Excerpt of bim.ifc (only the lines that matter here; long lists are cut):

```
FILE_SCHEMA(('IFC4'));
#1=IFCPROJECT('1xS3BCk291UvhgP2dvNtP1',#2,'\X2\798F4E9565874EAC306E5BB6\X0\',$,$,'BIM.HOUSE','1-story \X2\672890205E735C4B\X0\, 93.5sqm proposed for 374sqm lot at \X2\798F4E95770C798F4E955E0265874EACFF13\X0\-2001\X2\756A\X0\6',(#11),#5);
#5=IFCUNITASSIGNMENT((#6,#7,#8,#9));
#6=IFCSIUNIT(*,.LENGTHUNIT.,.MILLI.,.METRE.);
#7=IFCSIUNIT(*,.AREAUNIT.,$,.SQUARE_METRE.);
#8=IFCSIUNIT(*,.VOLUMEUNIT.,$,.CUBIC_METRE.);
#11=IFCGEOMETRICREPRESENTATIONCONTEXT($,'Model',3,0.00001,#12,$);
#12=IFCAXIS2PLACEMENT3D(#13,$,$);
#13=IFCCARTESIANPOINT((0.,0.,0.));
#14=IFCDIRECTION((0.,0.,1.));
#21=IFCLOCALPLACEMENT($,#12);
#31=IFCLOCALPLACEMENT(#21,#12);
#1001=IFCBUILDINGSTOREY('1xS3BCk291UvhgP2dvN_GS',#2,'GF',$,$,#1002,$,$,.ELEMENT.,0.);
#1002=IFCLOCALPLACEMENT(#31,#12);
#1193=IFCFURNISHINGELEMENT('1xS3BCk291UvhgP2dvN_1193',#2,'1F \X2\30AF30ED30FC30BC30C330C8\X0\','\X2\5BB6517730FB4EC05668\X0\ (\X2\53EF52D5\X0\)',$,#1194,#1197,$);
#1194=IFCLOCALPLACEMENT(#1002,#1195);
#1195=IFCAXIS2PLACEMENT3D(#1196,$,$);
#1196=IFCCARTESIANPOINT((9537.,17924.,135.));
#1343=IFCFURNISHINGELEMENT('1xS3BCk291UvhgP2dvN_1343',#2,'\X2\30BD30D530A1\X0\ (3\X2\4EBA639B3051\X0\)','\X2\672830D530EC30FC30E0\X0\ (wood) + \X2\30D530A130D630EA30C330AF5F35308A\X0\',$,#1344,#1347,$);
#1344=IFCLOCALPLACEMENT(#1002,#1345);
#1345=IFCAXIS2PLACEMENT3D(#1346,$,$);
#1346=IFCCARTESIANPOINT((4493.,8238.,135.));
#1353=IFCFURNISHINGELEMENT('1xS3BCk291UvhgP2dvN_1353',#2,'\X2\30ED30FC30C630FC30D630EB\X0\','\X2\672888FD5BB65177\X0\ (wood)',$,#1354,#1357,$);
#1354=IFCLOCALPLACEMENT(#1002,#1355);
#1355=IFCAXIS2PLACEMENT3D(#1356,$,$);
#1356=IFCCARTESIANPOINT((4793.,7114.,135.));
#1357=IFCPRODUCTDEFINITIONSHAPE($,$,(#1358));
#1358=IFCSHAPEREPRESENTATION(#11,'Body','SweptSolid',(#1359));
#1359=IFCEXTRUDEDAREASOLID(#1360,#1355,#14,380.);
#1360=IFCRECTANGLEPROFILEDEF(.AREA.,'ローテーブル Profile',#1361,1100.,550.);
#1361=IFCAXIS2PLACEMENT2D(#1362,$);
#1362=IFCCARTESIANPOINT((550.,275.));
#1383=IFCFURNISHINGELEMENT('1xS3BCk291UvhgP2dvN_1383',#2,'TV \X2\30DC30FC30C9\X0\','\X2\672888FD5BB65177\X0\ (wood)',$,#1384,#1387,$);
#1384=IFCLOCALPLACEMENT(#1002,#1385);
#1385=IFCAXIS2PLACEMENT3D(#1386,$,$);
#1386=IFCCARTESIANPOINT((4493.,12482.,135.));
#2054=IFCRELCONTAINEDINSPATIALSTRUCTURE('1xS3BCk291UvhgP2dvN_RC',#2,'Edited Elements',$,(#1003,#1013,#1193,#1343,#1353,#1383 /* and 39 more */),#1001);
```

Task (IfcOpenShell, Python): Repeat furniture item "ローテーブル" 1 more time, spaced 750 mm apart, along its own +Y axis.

```python
import ifcopenshell
import ifcopenshell.api.geometry
import ifcopenshell.api.root
import ifcopenshell.util.element
import ifcopenshell.util.placement

model = ifcopenshell.open("bim.ifc")


def reuse_history(source, copy):
    """copy_class also copies each property set's owner history, people and application; keep the originals."""
    for rel in copy.IsDefinedBy:
        if rel.is_a("IfcRelDefinesByProperties") and (history := rel.RelatingPropertyDefinition.OwnerHistory):
            rel.RelatingPropertyDefinition.OwnerHistory = source.OwnerHistory
            ifcopenshell.util.element.remove_deep2(model, history)


source = model.by_guid("1xS3BCk291UvhgP2dvN_1353")
base = ifcopenshell.util.placement.get_local_placement(source.ObjectPlacement)
step = base[:3, 1] * 750.0

for i in range(1, 2):
    copy = ifcopenshell.api.root.copy_class(model, product=source)
    copy.Representation = ifcopenshell.util.element.copy_deep(
        model, source.Representation, exclude=["IfcGeometricRepresentationContext", "IfcRepresentationMap"]
    )
    reuse_history(source, copy)
    matrix = base.copy()
    matrix[:3, 3] += i * step
    print("added at", matrix[:3, 3].round(3) + 0.0)
    ifcopenshell.api.geometry.edit_object_placement(model, product=copy, matrix=matrix, is_si=False)

model.write("bim_edited.ifc")
```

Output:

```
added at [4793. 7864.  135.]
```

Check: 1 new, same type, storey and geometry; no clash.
